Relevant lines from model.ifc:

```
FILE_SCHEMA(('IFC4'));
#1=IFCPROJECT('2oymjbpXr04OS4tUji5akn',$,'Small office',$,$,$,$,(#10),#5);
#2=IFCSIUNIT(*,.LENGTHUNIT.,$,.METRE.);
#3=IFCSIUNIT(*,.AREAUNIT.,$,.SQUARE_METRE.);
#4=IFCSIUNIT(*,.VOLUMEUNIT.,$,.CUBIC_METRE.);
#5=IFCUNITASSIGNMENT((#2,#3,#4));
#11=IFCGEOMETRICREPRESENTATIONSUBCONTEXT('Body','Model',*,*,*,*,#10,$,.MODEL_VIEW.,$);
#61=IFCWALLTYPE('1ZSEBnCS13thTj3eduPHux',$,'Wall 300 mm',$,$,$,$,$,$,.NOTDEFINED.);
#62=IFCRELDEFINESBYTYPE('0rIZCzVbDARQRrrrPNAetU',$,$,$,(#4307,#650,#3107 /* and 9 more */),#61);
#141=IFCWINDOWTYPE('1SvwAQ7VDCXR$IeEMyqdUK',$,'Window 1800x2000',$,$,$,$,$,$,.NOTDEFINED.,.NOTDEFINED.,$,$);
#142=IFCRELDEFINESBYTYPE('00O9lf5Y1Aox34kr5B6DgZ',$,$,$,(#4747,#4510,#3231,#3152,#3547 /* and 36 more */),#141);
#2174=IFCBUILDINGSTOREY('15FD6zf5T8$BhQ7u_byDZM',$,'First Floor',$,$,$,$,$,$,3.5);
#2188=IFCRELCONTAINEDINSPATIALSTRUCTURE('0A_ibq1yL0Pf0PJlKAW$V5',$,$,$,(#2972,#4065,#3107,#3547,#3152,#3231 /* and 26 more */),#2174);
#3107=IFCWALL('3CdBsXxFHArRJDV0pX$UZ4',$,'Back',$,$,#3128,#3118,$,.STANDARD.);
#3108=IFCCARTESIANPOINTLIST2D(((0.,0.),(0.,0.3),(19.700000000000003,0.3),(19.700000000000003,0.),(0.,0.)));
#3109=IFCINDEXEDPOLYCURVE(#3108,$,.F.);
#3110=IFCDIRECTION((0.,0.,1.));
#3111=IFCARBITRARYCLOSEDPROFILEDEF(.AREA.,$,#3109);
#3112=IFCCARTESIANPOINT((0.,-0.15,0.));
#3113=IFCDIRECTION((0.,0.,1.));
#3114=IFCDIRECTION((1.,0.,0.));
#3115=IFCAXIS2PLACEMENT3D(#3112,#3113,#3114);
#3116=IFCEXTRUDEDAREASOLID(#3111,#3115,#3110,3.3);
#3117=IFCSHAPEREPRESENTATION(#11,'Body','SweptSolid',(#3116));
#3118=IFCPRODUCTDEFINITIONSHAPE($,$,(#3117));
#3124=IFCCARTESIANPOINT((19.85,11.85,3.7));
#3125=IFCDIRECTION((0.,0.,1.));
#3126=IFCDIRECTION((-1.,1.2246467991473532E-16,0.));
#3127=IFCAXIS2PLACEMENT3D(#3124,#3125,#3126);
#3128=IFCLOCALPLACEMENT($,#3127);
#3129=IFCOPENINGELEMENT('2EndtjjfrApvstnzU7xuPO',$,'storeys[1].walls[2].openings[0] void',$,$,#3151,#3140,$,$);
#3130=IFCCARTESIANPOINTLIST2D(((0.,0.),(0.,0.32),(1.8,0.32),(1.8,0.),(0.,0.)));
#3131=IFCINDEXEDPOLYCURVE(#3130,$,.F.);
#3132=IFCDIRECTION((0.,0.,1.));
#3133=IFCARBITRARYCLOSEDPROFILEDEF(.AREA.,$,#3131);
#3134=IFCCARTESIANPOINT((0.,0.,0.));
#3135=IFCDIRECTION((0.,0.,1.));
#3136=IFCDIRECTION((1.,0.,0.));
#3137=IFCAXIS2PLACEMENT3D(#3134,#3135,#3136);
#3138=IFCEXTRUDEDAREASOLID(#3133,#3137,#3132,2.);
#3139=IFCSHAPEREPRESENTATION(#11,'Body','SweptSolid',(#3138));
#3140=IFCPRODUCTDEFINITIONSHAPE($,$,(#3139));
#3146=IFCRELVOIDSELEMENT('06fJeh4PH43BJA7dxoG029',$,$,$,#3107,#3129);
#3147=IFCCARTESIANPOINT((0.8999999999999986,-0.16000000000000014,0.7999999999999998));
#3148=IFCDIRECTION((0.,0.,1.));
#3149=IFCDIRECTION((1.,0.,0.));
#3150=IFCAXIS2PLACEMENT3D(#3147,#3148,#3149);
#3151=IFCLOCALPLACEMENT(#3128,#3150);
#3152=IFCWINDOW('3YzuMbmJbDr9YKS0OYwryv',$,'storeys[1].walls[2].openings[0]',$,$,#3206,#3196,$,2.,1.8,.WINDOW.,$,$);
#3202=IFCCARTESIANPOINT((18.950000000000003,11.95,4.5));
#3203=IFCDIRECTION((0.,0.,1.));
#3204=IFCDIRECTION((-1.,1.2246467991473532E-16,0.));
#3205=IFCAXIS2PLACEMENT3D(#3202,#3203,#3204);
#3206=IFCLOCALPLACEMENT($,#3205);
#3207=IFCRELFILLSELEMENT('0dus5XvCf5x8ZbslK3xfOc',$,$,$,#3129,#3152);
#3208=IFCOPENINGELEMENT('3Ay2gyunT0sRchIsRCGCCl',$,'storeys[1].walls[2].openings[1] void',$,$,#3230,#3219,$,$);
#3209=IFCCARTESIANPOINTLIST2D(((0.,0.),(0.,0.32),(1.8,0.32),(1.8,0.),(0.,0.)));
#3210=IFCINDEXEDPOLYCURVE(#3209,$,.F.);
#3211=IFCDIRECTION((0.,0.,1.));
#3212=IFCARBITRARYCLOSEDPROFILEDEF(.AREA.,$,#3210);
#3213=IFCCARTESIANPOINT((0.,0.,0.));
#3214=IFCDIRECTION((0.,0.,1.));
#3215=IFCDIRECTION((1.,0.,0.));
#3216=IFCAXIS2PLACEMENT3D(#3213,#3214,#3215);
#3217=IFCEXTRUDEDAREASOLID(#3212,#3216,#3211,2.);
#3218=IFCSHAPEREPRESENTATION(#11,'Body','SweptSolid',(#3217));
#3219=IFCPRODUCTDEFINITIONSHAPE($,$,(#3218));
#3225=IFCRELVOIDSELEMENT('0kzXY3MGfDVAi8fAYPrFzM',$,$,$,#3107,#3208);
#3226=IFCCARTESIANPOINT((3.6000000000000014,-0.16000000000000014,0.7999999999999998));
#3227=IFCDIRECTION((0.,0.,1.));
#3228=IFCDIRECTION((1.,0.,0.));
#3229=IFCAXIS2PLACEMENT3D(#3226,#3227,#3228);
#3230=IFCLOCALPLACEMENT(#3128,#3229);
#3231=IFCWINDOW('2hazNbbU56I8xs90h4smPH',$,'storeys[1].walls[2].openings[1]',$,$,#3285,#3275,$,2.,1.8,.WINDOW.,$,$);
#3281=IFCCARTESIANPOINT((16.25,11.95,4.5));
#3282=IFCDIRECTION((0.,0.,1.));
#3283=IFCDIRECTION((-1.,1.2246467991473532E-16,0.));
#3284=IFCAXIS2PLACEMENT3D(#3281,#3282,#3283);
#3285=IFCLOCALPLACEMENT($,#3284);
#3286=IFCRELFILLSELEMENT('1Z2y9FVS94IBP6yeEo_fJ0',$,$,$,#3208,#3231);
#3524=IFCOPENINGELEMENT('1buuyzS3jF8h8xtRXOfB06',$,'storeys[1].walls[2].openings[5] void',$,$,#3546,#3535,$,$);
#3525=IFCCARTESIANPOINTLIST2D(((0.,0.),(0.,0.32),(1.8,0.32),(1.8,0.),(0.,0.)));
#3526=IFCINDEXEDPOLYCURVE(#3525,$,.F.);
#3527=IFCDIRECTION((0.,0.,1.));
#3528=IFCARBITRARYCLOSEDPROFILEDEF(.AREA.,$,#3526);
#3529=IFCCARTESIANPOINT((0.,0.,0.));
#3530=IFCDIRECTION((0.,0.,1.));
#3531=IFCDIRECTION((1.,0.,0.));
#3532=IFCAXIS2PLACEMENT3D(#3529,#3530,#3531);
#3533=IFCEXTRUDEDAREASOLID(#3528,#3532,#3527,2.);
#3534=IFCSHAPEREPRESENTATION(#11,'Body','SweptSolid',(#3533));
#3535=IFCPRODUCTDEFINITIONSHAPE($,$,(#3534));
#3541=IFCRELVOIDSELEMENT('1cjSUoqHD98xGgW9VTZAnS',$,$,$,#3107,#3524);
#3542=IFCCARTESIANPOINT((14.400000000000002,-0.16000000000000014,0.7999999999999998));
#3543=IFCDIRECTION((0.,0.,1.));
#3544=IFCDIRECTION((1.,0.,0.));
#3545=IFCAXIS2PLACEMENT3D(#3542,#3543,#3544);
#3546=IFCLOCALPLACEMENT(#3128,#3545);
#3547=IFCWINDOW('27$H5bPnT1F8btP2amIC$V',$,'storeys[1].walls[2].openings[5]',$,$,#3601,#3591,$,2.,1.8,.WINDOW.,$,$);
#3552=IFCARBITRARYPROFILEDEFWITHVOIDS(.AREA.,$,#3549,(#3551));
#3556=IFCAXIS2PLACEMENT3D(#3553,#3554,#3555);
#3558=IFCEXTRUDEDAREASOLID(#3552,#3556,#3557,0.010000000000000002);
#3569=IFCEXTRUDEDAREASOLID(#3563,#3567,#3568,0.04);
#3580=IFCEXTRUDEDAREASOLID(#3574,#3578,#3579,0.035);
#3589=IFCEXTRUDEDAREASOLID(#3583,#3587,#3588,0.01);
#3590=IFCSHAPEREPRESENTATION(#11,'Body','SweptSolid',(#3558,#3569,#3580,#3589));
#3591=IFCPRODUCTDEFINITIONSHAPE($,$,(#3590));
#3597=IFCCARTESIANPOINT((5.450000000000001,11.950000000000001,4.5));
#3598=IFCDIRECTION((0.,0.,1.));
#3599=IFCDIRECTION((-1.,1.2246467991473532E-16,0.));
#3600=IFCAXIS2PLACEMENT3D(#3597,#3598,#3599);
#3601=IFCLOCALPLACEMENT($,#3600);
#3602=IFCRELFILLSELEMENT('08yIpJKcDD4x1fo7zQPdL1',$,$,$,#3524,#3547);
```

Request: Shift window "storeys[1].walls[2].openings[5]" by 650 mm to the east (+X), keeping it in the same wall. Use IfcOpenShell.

```python
import ifcopenshell
import ifcopenshell.api.geometry
import ifcopenshell.util.placement

model = ifcopenshell.open("model.ifc")

window = model.by_guid("27$H5bPnT1F8btP2amIC$V")
opening = window.FillsVoids[0].RelatingOpeningElement
wall = opening.VoidsElements[0].RelatingBuildingElement

wall_matrix = ifcopenshell.util.placement.get_local_placement(wall.ObjectPlacement)
shift = wall_matrix[:3, 0] * -0.65
before = ifcopenshell.util.placement.get_local_placement(window.ObjectPlacement)[:3, 3].copy()

# The window is not placed relative to its opening, so move both.
for product in (opening, window):
    matrix = ifcopenshell.util.placement.get_local_placement(product.ObjectPlacement)
    matrix[:3, 3] += shift
    ifcopenshell.api.geometry.edit_object_placement(model, product=product, matrix=matrix, is_si=False)

after = ifcopenshell.util.placement.get_local_placement(window.ObjectPlacement)[:3, 3]
print("window moved by", (after - before).round(3) + 0.0)

model.write("model-out.ifc")
```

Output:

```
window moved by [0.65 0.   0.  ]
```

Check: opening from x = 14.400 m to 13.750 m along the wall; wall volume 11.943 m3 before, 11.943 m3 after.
